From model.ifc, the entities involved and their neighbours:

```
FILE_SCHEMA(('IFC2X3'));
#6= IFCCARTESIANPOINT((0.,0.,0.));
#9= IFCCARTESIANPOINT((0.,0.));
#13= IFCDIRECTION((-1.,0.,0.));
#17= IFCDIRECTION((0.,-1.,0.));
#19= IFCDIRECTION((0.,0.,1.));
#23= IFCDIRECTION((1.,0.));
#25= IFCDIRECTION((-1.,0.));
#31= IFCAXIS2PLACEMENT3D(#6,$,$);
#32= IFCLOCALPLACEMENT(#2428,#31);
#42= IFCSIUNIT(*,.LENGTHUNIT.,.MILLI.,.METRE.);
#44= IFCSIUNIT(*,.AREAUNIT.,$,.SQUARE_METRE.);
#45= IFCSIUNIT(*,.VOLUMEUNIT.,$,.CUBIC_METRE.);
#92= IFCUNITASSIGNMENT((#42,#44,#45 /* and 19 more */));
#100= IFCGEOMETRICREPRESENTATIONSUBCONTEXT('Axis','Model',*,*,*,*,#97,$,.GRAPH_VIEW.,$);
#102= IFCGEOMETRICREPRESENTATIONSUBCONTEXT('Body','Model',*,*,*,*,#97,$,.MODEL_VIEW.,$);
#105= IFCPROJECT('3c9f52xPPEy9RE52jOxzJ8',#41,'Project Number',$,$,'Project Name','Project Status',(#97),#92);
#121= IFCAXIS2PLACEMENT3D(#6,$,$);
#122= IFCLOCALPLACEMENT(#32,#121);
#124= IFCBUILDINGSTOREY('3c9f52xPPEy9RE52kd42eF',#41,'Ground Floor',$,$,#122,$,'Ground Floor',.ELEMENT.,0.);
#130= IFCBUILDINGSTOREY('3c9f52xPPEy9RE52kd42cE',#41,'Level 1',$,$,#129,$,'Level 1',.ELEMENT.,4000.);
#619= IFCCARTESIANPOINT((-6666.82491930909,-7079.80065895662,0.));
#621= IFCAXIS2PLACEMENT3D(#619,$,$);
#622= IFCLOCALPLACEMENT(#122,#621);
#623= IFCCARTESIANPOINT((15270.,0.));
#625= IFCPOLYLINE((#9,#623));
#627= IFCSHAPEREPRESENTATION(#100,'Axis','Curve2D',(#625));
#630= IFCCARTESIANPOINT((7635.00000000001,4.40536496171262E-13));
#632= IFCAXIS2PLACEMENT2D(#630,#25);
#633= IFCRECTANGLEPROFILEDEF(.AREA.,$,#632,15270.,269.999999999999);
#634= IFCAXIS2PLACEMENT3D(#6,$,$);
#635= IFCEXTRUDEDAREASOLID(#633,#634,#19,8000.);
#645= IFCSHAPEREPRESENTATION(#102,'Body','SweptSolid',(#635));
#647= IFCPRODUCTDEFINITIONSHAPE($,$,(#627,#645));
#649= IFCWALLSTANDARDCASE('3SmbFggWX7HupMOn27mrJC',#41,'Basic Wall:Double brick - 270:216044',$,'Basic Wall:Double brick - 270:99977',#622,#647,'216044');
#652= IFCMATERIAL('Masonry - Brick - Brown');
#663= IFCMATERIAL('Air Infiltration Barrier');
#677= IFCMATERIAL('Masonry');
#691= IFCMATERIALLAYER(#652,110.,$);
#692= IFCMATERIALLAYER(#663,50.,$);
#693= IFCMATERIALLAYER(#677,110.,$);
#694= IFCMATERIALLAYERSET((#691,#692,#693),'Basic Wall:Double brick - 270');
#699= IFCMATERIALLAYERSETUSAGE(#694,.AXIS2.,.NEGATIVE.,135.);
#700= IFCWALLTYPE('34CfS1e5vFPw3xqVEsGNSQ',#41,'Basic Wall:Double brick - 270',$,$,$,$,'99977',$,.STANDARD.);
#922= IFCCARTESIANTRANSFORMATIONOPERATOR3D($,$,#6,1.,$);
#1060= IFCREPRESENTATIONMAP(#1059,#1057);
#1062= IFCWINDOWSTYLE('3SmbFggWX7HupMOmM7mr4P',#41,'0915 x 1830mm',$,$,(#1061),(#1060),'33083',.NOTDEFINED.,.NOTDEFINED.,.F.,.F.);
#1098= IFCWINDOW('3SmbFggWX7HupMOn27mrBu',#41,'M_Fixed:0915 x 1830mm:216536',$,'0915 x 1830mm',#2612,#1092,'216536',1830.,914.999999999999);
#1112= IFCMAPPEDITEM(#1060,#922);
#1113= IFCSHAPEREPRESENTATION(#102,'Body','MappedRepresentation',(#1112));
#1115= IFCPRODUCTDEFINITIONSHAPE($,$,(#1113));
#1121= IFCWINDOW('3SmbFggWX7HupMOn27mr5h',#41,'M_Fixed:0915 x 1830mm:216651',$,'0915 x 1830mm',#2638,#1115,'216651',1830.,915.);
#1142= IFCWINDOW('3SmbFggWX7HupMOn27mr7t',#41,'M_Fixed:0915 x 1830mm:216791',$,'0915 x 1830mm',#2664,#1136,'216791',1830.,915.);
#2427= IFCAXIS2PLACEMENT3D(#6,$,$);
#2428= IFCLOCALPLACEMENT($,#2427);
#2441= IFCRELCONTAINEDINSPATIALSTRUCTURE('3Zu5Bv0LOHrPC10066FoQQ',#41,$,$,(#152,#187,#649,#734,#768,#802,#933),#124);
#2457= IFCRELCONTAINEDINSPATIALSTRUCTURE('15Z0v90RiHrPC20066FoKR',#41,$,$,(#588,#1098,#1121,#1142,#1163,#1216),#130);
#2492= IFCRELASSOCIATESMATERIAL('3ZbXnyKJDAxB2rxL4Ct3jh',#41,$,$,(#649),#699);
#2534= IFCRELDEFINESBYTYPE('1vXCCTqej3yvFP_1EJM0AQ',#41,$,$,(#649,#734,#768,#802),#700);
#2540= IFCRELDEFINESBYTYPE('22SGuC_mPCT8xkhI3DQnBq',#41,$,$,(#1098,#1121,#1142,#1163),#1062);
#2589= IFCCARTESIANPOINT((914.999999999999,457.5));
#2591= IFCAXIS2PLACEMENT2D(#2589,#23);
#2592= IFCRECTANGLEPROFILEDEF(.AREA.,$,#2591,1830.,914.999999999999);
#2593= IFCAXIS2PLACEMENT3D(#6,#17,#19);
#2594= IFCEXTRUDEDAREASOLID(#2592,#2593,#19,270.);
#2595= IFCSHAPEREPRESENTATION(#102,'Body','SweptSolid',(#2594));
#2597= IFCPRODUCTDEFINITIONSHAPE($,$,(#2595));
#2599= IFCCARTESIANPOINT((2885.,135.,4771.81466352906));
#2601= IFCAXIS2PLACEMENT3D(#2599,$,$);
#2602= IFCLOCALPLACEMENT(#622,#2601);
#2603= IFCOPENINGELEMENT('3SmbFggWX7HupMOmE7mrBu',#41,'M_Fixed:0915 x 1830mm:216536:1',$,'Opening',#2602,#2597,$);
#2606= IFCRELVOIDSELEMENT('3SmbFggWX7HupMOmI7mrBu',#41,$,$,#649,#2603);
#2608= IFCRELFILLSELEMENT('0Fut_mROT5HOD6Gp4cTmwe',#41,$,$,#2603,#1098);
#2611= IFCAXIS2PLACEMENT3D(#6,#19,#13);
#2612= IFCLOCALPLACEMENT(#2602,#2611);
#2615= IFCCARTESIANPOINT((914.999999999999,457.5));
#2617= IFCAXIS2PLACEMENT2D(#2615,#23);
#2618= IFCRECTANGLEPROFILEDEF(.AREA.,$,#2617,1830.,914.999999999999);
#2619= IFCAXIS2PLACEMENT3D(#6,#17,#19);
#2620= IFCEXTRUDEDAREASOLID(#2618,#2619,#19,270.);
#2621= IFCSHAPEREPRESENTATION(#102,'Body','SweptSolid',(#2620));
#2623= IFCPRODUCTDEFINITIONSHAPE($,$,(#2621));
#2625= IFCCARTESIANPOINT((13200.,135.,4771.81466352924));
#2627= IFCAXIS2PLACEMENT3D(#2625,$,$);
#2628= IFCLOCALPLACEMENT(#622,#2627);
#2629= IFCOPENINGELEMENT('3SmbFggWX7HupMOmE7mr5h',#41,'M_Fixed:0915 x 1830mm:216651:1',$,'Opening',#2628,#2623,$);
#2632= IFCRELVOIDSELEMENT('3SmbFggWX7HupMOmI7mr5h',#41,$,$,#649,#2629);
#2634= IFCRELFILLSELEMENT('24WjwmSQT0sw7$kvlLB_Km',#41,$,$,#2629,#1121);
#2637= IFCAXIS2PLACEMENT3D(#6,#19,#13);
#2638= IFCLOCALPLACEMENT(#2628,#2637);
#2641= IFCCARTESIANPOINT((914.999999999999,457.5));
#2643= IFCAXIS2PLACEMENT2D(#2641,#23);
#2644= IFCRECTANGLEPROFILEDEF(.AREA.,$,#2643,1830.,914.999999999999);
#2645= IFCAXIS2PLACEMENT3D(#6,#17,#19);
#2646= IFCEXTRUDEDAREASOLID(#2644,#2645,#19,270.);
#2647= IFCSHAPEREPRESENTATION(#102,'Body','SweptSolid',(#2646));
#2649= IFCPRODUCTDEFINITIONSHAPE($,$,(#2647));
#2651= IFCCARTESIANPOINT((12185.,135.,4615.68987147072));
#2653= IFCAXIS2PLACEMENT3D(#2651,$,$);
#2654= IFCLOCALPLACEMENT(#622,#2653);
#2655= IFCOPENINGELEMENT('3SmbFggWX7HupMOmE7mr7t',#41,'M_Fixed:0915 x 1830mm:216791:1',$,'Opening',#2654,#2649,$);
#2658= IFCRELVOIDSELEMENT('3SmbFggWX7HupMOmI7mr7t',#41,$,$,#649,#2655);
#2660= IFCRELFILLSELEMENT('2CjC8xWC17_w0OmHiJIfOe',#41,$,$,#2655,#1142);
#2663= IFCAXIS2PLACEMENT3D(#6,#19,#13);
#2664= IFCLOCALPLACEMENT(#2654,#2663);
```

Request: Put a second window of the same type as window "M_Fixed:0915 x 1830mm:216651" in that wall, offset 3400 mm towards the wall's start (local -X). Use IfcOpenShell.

```python
import ifcopenshell
import ifcopenshell.api.feature
import ifcopenshell.api.geometry
import ifcopenshell.api.root
import ifcopenshell.geom
import ifcopenshell.util.element
import ifcopenshell.util.placement
import ifcopenshell.util.shape
import ifcopenshell.util.unit

model = ifcopenshell.open("model.ifc")
unit_scale = ifcopenshell.util.unit.calculate_unit_scale(model)
settings = ifcopenshell.geom.settings()


def volume(element):
    """Net volume in cubic metres, openings subtracted."""
    shape = ifcopenshell.geom.create_shape(settings, element)
    return ifcopenshell.util.shape.get_volume(shape.geometry)


def reuse_history(source, copy):
    """copy_class also copies each property set's owner history, people and application; keep the originals."""
    for rel in copy.IsDefinedBy:
        if rel.is_a("IfcRelDefinesByProperties") and (history := rel.RelatingPropertyDefinition.OwnerHistory):
            rel.RelatingPropertyDefinition.OwnerHistory = source.OwnerHistory
            ifcopenshell.util.element.remove_deep2(model, history)


window = model.by_id(1121)
opening = window.FillsVoids[0].RelatingOpeningElement
wall = opening.VoidsElements[0].RelatingBuildingElement
before = volume(wall)
shift = ifcopenshell.util.placement.get_local_placement(wall.ObjectPlacement)[:3, 0] * -3.4 / unit_scale

# copy_class copies the void relationship, type, container and properties, but no geometry.
new_opening = ifcopenshell.api.root.copy_class(model, product=opening)
new_opening.Representation = ifcopenshell.util.element.copy_deep(
    model, opening.Representation, exclude=["IfcGeometricRepresentationContext", "IfcRepresentationMap"]
)
new_opening.Name = "M_Fixed:0915 x 1830mm"
new_window = ifcopenshell.api.root.copy_class(model, product=window)
new_window.Representation = ifcopenshell.util.element.copy_deep(
    model, window.Representation, exclude=["IfcGeometricRepresentationContext", "IfcRepresentationMap"]
)
new_window.Name = "M_Fixed:0915 x 1830mm"
new_window.Tag = None
reuse_history(window, new_window)
fills = ifcopenshell.api.feature.add_filling(model, opening=new_opening, element=new_window)
fills.OwnerHistory = new_window.OwnerHistory  # required in IFC2X3

for old, new in ((opening, new_opening), (window, new_window)):
    matrix = ifcopenshell.util.placement.get_local_placement(old.ObjectPlacement)
    matrix[:3, 3] += shift
    ifcopenshell.api.geometry.edit_object_placement(model, product=new, matrix=matrix, is_si=False)

after = volume(wall)

print(f"wall volume {before:.3f} -> {after:.3f} m3")

model.write("model_updated.ifc")
```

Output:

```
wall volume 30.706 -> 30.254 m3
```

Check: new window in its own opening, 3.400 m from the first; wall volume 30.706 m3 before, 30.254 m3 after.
